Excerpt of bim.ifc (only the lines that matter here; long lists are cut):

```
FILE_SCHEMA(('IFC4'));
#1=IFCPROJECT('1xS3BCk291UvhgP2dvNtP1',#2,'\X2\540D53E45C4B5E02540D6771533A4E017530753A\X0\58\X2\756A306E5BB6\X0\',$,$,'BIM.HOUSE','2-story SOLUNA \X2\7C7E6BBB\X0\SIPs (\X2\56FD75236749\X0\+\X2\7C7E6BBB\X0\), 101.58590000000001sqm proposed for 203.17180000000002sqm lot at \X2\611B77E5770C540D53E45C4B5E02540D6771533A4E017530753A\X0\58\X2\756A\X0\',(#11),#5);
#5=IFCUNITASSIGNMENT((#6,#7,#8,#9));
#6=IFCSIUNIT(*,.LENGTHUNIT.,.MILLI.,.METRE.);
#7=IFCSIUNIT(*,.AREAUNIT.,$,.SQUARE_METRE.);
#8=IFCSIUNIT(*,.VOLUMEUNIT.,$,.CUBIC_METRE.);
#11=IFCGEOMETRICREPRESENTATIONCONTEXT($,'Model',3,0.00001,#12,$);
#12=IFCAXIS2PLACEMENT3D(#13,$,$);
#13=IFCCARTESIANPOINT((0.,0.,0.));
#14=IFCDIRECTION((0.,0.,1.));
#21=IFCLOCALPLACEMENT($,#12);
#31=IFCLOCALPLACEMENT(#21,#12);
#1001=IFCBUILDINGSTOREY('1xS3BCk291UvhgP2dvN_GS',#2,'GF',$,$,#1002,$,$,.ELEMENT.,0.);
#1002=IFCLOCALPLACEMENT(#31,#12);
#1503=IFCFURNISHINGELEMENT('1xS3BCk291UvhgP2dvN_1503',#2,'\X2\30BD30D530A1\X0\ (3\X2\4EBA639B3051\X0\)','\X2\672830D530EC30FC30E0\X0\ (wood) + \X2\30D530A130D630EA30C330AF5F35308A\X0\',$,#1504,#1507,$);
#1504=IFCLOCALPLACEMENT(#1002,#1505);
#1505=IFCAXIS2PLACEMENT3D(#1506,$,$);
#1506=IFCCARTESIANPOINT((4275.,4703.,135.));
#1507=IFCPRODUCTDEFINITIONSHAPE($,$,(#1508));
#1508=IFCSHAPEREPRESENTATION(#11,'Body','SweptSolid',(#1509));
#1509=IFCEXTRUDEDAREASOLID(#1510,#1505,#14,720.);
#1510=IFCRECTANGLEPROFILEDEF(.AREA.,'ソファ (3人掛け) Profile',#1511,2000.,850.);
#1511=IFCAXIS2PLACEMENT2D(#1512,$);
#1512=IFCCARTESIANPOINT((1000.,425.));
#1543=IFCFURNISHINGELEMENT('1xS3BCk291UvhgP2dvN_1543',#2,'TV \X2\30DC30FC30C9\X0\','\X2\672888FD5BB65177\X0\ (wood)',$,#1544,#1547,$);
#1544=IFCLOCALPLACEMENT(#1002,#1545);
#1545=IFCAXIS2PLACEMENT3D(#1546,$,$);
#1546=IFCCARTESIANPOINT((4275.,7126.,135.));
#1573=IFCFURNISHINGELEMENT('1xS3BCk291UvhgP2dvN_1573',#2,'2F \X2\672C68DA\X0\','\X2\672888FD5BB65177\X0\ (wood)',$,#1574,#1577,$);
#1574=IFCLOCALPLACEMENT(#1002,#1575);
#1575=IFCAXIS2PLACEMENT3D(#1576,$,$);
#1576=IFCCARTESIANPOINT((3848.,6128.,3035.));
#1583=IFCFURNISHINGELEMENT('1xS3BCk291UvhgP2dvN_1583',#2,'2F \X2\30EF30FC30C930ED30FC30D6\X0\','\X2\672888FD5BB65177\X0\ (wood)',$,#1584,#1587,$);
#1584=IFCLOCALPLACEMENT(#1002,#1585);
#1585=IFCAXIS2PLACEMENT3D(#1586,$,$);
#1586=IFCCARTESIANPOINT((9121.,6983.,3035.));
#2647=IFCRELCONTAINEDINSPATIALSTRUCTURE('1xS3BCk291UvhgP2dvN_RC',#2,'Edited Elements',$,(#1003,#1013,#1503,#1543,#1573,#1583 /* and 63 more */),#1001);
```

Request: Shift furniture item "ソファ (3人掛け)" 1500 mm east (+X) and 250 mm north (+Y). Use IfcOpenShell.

```python
import ifcopenshell
import ifcopenshell.api.geometry
import ifcopenshell.util.placement

model = ifcopenshell.open("bim.ifc")

item = model.by_id(1503)
matrix = ifcopenshell.util.placement.get_local_placement(item.ObjectPlacement)
matrix[0, 3] += 1500.0
matrix[1, 3] += 250.0
ifcopenshell.api.geometry.edit_object_placement(model, product=item, matrix=matrix, is_si=False)

print(ifcopenshell.util.placement.get_local_placement(item.ObjectPlacement).round(3) + 0.0)

model.write("bim_v2.ifc")
```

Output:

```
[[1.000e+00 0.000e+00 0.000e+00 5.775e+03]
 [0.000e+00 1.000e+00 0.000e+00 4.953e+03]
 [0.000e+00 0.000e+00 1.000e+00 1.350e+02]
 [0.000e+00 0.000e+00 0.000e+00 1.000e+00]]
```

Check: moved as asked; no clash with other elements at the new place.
